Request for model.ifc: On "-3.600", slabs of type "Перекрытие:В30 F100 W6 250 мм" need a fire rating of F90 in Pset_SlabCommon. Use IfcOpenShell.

First a look at what the model holds.

```python
import ifcopenshell
import ifcopenshell.util.element

model = ifcopenshell.open("model.ifc")
print(model.schema)
storey = next(s for s in model.by_type("IfcBuildingStorey") if s.Name == "-3.600")
slabs = [e for e in ifcopenshell.util.element.get_decomposition(storey) if e.is_a("IfcSlab")]
seen = {}
for e in slabs:
    element_type = ifcopenshell.util.element.get_type(e)
    key = (element_type.Name if element_type != e and element_type else None, ifcopenshell.util.element.get_pset(e, "Pset_SlabCommon", "FireRating"))
    seen[key] = seen.get(key, 0) + 1
for (name, value), count in sorted(seen.items(), key=str):
    print(count, "x", name, "|", value)
```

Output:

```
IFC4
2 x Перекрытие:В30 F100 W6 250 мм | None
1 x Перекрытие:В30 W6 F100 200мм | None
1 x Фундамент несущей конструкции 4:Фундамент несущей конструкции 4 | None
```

```python
import ifcopenshell
import ifcopenshell.api.pset
import ifcopenshell.util.element

model = ifcopenshell.open("model.ifc")

storey = next(s for s in model.by_type("IfcBuildingStorey") if s.Name == "-3.600")
slabs = [e for e in ifcopenshell.util.element.get_decomposition(storey) if e.is_a("IfcSlab")]

count = 0
for e in slabs:
    element_type = ifcopenshell.util.element.get_type(e)
    if element_type in (None, e) or element_type.Name != "Перекрытие:В30 F100 W6 250 мм":
        continue
    # add_pset returns the element's existing set when there is one.
    pset = ifcopenshell.api.pset.add_pset(model, product=e, name="Pset_SlabCommon")
    ifcopenshell.api.pset.edit_pset(model, pset=pset, properties={"FireRating": "F90"})
    count += 1

print(count, "slabs updated")

model.write("model_rev.ifc")
```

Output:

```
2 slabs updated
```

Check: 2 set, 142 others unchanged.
